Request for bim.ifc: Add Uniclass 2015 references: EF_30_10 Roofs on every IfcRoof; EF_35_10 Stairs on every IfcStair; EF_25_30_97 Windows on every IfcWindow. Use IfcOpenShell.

First a look at what the model holds.

```python
import ifcopenshell

model = ifcopenshell.open("bim.ifc")
print(model.schema)
print("classifications:", [c.Name for c in model.by_type("IfcClassification")])
for ifc_class in ("IfcDoor", "IfcRoof", "IfcStair", "IfcWall", "IfcWindow"):
    print(ifc_class, len(model.by_type(ifc_class)))
```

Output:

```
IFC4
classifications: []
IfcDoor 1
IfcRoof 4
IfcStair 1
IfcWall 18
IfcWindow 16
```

```python
import ifcopenshell
import ifcopenshell.api.classification

model = ifcopenshell.open("bim.ifc")

system = ifcopenshell.api.classification.add_classification(model, classification="Uniclass 2015")

codes = {
    "IfcRoof": ("EF_30_10", "Roofs"),
    "IfcStair": ("EF_35_10", "Stairs"),
    "IfcWindow": ("EF_25_30_97", "Windows"),
}
for ifc_class, (code, name) in codes.items():
    products = model.by_type(ifc_class)
    ifcopenshell.api.classification.add_reference(
        model, products=products, classification=system, identification=code, name=name
    )
    print(code, len(products))

model.write("bim_rev.ifc")
```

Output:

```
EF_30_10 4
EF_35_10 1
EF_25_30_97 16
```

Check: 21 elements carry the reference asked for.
